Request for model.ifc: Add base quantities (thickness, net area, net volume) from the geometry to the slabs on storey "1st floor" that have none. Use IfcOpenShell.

First a look at what the model holds.

```python
import ifcopenshell
import ifcopenshell.util.element
import ifcopenshell.util.unit

model = ifcopenshell.open("model.ifc")
print(model.schema)
for unit_type in ("LENGTHUNIT", "AREAUNIT", "VOLUMEUNIT"):
    print(unit_type, ifcopenshell.util.unit.calculate_unit_scale(model, unit_type))
storey = next(s for s in model.by_type("IfcBuildingStorey") if s.Name == "1st floor")
slabs = [e for e in ifcopenshell.util.element.get_decomposition(storey) if e.is_a("IfcSlab")]
for e in sorted(slabs, key=lambda e: e.id()):
    print(e.id(), e.is_a(), e.Name, list(ifcopenshell.util.element.get_psets(e, qtos_only=True)), sep=" | ")
```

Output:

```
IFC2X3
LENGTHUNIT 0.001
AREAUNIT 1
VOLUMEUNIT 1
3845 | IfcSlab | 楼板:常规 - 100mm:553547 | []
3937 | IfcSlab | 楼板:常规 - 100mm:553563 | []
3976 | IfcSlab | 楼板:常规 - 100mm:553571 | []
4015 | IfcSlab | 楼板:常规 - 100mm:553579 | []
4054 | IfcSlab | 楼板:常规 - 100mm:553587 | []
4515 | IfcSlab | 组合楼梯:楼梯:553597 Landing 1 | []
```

```python
import ifcopenshell
import ifcopenshell.api.pset
import ifcopenshell.geom
import ifcopenshell.util.element
import ifcopenshell.util.shape
import ifcopenshell.util.unit

model = ifcopenshell.open("model.ifc")
unit_scale = ifcopenshell.util.unit.calculate_unit_scale(model)
area_scale = ifcopenshell.util.unit.calculate_unit_scale(model, "AREAUNIT")
volume_scale = ifcopenshell.util.unit.calculate_unit_scale(model, "VOLUMEUNIT")
settings = ifcopenshell.geom.settings()

storey = next(s for s in model.by_type("IfcBuildingStorey") if s.Name == "1st floor")
slabs = [e for e in ifcopenshell.util.element.get_decomposition(storey) if e.is_a("IfcSlab")]

for e in sorted(slabs, key=lambda e: e.id()):
    if ifcopenshell.util.element.get_psets(e, qtos_only=True, should_inherit=False):
        continue
    # Geometry comes back in metres, in the element's own axes.
    shape = ifcopenshell.geom.create_shape(settings, e)
    values = {
        "Width": ifcopenshell.util.shape.get_z(shape.geometry) / unit_scale,
        "NetArea": ifcopenshell.util.shape.get_footprint_area(shape.geometry) / area_scale,
        "NetVolume": ifcopenshell.util.shape.get_volume(shape.geometry) / volume_scale,
    }
    qto = ifcopenshell.api.pset.add_qto(model, product=e, name="BaseQuantities")
    ifcopenshell.api.pset.edit_qto(model, qto=qto, properties=values)
    print(e.id(), {k: round(v, 3) for k, v in values.items()})

model.write("model_rev.ifc")
```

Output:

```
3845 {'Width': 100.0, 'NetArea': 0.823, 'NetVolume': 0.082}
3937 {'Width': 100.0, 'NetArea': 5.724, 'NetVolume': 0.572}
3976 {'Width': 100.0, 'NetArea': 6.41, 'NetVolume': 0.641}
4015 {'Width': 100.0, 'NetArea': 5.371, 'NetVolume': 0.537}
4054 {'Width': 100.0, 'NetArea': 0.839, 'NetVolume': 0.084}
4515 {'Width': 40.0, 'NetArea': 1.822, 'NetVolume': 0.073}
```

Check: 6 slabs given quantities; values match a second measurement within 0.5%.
